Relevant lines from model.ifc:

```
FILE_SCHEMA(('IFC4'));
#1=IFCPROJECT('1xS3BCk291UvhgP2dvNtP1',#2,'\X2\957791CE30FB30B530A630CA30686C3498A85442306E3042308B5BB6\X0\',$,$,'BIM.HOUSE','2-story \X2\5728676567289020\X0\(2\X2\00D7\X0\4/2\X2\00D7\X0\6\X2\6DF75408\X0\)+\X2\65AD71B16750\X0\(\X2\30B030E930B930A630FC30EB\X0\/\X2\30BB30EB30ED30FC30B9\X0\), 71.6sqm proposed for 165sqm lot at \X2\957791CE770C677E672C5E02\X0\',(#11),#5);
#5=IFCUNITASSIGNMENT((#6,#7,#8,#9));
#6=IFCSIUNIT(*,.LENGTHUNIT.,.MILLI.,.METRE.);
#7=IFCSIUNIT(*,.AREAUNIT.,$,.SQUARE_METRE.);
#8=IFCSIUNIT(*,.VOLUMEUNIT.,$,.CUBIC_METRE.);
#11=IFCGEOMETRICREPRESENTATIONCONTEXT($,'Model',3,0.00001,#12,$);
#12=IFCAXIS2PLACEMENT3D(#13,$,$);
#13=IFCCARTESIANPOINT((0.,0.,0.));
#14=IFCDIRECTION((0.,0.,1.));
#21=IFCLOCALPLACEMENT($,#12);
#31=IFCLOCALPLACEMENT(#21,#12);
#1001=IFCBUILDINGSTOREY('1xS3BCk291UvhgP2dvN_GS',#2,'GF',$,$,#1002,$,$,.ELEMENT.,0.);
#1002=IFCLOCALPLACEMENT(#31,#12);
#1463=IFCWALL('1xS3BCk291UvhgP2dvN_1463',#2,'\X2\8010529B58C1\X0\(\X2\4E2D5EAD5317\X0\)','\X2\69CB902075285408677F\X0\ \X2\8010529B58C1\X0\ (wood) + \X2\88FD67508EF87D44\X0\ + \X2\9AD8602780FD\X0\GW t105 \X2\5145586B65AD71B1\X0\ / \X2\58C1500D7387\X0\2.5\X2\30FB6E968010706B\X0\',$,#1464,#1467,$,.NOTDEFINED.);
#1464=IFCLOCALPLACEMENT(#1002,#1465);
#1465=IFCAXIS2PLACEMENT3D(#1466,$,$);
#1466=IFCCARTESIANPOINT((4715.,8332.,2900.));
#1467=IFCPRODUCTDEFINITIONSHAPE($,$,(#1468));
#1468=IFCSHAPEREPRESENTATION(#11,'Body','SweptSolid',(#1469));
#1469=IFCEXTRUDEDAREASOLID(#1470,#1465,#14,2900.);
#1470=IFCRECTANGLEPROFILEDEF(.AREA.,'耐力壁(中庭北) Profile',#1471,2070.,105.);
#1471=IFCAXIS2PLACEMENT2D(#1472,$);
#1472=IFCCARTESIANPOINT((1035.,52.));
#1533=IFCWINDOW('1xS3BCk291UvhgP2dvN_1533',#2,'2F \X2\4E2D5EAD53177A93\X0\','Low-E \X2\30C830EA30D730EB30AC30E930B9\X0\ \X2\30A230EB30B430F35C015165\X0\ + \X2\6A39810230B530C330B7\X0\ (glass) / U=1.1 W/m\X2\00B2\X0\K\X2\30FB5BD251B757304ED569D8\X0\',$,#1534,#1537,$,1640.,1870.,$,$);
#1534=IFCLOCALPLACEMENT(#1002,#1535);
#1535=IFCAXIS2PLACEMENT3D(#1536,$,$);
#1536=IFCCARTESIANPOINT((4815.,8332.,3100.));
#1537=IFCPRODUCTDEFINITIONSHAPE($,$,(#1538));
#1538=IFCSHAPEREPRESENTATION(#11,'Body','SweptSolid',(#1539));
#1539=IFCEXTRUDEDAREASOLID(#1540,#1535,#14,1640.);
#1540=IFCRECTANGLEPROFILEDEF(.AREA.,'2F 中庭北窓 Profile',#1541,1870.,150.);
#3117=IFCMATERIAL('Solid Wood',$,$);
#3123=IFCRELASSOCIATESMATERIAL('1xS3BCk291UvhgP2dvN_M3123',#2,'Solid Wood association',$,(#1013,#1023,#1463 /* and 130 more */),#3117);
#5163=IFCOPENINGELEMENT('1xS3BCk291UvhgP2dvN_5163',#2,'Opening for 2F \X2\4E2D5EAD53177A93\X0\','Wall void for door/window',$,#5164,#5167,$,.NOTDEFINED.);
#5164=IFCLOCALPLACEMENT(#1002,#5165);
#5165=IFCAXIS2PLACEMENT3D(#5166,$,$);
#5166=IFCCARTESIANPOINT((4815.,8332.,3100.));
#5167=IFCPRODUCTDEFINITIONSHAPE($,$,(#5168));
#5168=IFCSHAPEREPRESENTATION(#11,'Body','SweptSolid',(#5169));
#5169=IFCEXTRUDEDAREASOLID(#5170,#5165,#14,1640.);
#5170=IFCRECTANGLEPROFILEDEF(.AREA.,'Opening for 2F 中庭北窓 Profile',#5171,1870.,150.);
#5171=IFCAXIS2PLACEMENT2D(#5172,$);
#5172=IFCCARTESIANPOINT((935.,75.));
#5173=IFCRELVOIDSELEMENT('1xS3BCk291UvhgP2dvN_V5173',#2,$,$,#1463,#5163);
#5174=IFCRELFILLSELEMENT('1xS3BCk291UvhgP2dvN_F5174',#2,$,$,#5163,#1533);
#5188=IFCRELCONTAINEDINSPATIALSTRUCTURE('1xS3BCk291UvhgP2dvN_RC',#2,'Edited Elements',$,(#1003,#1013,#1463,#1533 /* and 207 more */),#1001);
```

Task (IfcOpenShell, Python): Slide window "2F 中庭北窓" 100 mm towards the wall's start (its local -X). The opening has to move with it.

```python
import ifcopenshell
import ifcopenshell.api.geometry
import ifcopenshell.util.placement
import ifcopenshell.util.unit

model = ifcopenshell.open("model.ifc")
unit_scale = ifcopenshell.util.unit.calculate_unit_scale(model)

window = model.by_guid("1xS3BCk291UvhgP2dvN_1533")
opening = window.FillsVoids[0].RelatingOpeningElement
wall = opening.VoidsElements[0].RelatingBuildingElement

wall_matrix = ifcopenshell.util.placement.get_local_placement(wall.ObjectPlacement)
shift = wall_matrix[:3, 0] * -0.1 / unit_scale
before = ifcopenshell.util.placement.get_local_placement(window.ObjectPlacement)[:3, 3].copy()

# The window is not placed relative to its opening, so move both.
for product in (opening, window):
    matrix = ifcopenshell.util.placement.get_local_placement(product.ObjectPlacement)
    matrix[:3, 3] += shift
    ifcopenshell.api.geometry.edit_object_placement(model, product=product, matrix=matrix, is_si=False)

after = ifcopenshell.util.placement.get_local_placement(window.ObjectPlacement)[:3, 3]
print("window moved by", (after - before).round(3) + 0.0)

model.write("model_edited.ifc")
```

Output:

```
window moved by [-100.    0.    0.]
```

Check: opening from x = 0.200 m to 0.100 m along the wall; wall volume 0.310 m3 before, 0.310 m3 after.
